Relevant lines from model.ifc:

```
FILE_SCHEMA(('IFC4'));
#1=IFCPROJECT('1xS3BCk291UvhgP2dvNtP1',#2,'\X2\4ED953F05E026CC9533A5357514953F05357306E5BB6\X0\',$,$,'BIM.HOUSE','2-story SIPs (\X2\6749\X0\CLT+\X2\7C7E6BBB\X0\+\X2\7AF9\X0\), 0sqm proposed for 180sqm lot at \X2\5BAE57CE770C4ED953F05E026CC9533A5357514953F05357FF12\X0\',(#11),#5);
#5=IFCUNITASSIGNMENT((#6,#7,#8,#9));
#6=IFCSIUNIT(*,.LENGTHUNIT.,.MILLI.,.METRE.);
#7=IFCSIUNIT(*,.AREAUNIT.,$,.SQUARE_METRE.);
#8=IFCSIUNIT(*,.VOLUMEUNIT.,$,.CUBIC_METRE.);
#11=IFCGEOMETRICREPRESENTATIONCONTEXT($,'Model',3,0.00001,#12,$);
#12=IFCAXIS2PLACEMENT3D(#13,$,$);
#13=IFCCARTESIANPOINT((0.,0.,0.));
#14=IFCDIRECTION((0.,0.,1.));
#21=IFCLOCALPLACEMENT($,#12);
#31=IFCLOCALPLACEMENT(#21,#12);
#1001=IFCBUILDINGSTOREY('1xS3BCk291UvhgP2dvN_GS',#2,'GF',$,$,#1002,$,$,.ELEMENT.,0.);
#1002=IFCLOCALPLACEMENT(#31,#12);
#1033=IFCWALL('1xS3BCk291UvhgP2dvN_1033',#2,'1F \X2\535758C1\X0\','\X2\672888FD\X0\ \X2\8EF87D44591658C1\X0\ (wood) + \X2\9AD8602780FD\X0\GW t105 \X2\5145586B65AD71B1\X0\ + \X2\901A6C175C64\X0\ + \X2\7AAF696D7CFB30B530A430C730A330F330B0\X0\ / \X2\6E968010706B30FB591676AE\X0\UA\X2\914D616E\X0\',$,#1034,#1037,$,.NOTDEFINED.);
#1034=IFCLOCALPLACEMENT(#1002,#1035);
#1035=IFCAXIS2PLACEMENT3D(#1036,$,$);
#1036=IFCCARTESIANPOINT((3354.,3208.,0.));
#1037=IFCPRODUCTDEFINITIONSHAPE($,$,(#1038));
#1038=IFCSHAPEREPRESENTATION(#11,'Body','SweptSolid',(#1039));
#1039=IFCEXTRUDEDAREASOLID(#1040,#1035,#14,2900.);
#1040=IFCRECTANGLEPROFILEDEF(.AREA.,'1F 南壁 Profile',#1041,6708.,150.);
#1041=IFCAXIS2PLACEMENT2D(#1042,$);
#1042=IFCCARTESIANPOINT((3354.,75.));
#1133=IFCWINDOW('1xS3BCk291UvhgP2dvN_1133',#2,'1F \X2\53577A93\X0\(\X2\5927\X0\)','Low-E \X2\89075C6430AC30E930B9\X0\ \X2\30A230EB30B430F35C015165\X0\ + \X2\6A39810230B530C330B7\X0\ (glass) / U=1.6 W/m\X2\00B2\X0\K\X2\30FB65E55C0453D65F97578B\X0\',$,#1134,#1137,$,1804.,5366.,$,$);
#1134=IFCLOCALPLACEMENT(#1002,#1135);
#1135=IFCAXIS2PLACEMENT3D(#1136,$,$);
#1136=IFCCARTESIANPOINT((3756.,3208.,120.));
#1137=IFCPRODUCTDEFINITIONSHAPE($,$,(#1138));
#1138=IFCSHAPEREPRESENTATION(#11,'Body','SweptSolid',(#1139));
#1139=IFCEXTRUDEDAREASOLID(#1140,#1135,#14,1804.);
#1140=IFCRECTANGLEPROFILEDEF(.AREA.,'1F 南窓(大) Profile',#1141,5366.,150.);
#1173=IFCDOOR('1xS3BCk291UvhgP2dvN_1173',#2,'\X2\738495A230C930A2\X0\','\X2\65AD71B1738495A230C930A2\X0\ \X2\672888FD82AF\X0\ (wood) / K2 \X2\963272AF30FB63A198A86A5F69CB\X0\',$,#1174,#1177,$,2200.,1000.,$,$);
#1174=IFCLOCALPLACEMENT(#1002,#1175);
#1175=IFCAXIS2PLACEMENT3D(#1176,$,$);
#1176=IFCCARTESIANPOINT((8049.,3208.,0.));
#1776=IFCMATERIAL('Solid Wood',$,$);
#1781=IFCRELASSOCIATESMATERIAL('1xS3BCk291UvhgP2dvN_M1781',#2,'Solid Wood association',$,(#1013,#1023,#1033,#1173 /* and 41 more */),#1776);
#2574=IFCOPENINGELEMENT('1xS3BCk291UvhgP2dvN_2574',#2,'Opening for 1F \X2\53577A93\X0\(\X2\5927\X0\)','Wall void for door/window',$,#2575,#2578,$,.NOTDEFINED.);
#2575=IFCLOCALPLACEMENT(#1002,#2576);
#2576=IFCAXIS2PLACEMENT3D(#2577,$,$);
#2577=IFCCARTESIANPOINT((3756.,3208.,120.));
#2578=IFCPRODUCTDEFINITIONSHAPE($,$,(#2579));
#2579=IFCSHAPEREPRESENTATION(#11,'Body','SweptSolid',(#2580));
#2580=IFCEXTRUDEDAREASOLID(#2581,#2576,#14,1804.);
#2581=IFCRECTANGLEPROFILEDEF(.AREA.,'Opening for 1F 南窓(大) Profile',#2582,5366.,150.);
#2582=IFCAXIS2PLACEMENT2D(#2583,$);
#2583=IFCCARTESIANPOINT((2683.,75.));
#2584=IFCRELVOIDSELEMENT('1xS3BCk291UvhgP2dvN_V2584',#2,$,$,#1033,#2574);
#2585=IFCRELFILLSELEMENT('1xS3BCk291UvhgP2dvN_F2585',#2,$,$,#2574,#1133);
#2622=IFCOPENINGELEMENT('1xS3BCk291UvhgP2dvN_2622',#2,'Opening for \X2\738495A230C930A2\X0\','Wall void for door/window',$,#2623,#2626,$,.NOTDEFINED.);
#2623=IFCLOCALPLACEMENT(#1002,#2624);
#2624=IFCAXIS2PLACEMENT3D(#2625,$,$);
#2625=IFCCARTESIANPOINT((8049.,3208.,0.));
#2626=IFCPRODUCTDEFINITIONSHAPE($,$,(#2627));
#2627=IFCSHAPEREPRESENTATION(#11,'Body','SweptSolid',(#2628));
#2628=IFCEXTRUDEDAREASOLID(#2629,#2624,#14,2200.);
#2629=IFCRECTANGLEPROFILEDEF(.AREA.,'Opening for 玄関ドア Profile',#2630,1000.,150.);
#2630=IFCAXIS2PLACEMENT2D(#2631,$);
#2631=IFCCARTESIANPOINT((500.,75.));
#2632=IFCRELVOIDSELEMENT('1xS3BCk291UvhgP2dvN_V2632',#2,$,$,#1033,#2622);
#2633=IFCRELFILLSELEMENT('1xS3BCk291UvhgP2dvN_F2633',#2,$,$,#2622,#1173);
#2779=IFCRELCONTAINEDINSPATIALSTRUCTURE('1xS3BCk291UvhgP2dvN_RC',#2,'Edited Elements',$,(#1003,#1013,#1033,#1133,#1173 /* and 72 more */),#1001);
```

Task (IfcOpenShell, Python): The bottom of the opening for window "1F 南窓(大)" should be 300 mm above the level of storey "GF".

```python
import numpy as np
import ifcopenshell
import ifcopenshell.api.geometry
import ifcopenshell.geom
import ifcopenshell.util.element
import ifcopenshell.util.placement
import ifcopenshell.util.shape
import ifcopenshell.util.unit

model = ifcopenshell.open("model.ifc")
unit_scale = ifcopenshell.util.unit.calculate_unit_scale(model)

window = model.by_guid("1xS3BCk291UvhgP2dvN_1133")
opening = window.FillsVoids[0].RelatingOpeningElement
storey = ifcopenshell.util.element.get_container(window, ifc_class="IfcBuildingStorey")
level = ifcopenshell.util.placement.get_local_placement(storey.ObjectPlacement)[2, 3]

# The opening's origin need not be at the sill, so measure its lowest point.
shape = ifcopenshell.geom.create_shape(ifcopenshell.geom.settings(), opening)
bottom = ifcopenshell.util.shape.get_shape_bottom_elevation(shape, shape.geometry) / unit_scale
dz = level + 300.0 - bottom

shift = np.array([0.0, 0.0, dz])
# The window is not placed relative to its opening, so move both.
for product in (opening, window):
    matrix = ifcopenshell.util.placement.get_local_placement(product.ObjectPlacement)
    matrix[:3, 3] += shift
    ifcopenshell.api.geometry.edit_object_placement(model, product=product, matrix=matrix, is_si=False)

print(f"moved by {dz * unit_scale:+.3f} m")

model.write("model_edited.ifc")
```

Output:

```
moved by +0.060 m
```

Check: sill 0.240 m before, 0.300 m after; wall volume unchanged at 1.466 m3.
